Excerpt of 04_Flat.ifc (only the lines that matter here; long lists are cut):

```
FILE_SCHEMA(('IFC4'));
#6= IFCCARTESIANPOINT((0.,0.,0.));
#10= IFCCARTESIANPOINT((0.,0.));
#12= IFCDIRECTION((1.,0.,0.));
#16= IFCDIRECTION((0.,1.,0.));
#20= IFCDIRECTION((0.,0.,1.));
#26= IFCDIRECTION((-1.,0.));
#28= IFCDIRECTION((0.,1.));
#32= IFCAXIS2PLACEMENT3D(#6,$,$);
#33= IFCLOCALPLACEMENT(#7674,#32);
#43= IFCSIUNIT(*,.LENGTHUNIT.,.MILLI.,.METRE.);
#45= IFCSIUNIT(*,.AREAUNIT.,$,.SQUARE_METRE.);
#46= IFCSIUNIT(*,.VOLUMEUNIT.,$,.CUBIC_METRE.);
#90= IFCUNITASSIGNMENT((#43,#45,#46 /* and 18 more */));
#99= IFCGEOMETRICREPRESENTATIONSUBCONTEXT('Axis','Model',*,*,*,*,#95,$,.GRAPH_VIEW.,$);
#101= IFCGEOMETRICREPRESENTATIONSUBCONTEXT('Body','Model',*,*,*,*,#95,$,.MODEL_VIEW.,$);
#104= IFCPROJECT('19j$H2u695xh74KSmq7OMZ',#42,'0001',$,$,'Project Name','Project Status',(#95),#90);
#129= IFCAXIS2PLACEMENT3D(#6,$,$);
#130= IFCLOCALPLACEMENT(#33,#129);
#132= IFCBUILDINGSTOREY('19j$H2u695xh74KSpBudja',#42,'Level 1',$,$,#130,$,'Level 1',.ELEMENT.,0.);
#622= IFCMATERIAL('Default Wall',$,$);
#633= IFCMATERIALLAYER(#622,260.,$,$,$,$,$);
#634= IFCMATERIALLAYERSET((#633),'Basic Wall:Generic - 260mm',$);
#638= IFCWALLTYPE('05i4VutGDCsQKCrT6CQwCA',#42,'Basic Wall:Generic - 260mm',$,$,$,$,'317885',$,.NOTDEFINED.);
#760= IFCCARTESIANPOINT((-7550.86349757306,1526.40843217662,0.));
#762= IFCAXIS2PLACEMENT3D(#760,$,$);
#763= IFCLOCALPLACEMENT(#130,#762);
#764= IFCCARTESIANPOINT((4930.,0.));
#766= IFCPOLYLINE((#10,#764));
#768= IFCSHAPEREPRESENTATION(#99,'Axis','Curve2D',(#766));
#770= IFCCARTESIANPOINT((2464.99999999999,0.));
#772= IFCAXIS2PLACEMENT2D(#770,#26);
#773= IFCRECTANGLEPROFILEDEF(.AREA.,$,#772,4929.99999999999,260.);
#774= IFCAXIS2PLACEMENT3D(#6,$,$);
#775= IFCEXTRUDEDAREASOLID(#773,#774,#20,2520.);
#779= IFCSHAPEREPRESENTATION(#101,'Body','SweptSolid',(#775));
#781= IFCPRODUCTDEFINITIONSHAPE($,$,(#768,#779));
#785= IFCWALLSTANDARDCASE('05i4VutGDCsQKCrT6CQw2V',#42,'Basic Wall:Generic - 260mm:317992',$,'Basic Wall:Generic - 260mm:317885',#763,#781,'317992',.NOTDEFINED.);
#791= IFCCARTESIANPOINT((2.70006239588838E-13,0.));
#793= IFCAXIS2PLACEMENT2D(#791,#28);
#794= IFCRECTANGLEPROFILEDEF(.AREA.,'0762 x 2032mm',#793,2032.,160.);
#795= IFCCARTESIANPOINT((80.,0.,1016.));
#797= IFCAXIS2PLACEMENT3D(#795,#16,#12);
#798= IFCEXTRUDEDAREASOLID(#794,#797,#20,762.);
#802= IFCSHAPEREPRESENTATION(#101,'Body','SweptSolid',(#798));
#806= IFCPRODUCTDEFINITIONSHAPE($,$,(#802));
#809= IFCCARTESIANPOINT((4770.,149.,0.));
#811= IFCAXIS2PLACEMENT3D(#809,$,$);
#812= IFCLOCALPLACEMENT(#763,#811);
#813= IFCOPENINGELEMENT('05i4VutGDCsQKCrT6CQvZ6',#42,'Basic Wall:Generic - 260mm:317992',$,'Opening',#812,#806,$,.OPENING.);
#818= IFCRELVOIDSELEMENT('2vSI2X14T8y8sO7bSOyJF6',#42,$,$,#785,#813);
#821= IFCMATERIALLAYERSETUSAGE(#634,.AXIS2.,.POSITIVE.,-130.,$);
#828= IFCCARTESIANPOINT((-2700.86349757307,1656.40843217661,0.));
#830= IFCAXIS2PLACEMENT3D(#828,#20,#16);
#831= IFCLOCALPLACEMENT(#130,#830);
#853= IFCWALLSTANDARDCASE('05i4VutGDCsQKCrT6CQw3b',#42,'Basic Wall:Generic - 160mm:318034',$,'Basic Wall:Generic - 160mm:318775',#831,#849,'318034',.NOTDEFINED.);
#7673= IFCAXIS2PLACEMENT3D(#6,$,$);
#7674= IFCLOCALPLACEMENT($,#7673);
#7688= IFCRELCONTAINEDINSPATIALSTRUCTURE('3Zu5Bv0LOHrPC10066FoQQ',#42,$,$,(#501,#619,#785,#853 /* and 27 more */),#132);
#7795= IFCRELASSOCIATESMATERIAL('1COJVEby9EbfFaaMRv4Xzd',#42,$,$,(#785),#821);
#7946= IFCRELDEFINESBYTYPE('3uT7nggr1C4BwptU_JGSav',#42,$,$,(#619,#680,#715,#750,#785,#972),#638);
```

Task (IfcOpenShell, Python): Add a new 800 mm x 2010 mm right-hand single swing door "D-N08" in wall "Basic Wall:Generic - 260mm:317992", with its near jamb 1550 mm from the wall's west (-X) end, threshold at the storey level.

```python
import numpy as np
import ifcopenshell
import ifcopenshell.api.feature
import ifcopenshell.api.geometry
import ifcopenshell.api.root
import ifcopenshell.api.spatial
import ifcopenshell.geom
import ifcopenshell.util.element
import ifcopenshell.util.placement
import ifcopenshell.util.representation
import ifcopenshell.util.shape
import ifcopenshell.util.unit

model = ifcopenshell.open("04_Flat.ifc")
unit_scale = ifcopenshell.util.unit.calculate_unit_scale(model)
settings = ifcopenshell.geom.settings()


def volume(element):
    """Net volume in cubic metres, openings subtracted."""
    shape = ifcopenshell.geom.create_shape(settings, element)
    return ifcopenshell.util.shape.get_volume(shape.geometry)


wall = model.by_id(785)
storey = ifcopenshell.util.element.get_container(wall, ifc_class="IfcBuildingStorey")
context = ifcopenshell.util.representation.get_context(model, "Model", "Body", "MODEL_VIEW")
before = volume(wall)

width, height, from_end, sill = 0.8, 2.01, 1.55, 0.0  # metres

# The wall runs along its own X axis, and the end named is its -X end.
wall_shape = ifcopenshell.geom.create_shape(settings, wall)
x, y, z = ifcopenshell.util.shape.get_vertices(wall_shape.geometry).T
start = x.min() + from_end
face, thickness = float(y.min()), float(y.max() - y.min())
wall_matrix = ifcopenshell.util.placement.get_local_placement(wall.ObjectPlacement)
level = ifcopenshell.util.placement.get_local_placement(storey.ObjectPlacement)[2, 3]


def in_wall(x, y):
    """Placement at x, y metres in the wall's axes, at sill height."""
    matrix = wall_matrix.copy()
    matrix[:, 3] = wall_matrix @ np.array([x / unit_scale, y / unit_scale, 0.0, 1.0])
    matrix[2, 3] = level + sill / unit_scale
    return matrix


# Opening: a box that overshoots both wall faces by 50 mm.
opening = ifcopenshell.api.root.create_entity(model, ifc_class="IfcOpeningElement", predefined_type="OPENING")
box = ifcopenshell.api.geometry.add_wall_representation(
    model, context=context, length=width, height=height, thickness=thickness + 0.1
)
ifcopenshell.api.geometry.assign_representation(model, product=opening, representation=box)
ifcopenshell.api.geometry.edit_object_placement(model, product=opening, matrix=in_wall(start, face - 0.05), is_si=False)
ifcopenshell.api.feature.add_feature(model, feature=opening, element=wall)

door = ifcopenshell.api.root.create_entity(model, ifc_class="IfcDoor", name="D-N08", predefined_type="DOOR")
door.OverallWidth, door.OverallHeight = width / unit_scale, height / unit_scale
door.OperationType = "SINGLE_SWING_RIGHT"
body = ifcopenshell.api.geometry.add_door_representation(
    model,
    context=context,
    overall_width=door.OverallWidth,
    overall_height=door.OverallHeight,
    operation_type="SINGLE_SWING_RIGHT",
    lining_properties={"LiningDepth": thickness / unit_scale, "ThresholdDepth": thickness / unit_scale},
)
ifcopenshell.api.geometry.assign_representation(model, product=door, representation=body)
ifcopenshell.api.spatial.assign_container(model, products=[door], relating_structure=storey)
ifcopenshell.api.feature.add_filling(model, opening=opening, element=door)

# The lining spans the wall, so the door starts at the wall face.
ifcopenshell.api.geometry.edit_object_placement(model, product=door, matrix=in_wall(start, face), is_si=False)

after = volume(wall)

print(f"wall volume {before:.3f} -> {after:.3f} m3")

model.write("04_Flat_rev.ifc")
```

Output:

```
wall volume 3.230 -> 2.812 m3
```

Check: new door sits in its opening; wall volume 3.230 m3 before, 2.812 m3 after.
